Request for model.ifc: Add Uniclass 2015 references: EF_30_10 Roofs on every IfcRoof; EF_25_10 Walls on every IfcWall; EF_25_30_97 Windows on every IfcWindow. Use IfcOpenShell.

First a look at what the model holds.

```python
import ifcopenshell

model = ifcopenshell.open("model.ifc")
print(model.schema)
print("classifications:", [c.Name for c in model.by_type("IfcClassification")])
for ifc_class in ("IfcDoor", "IfcRoof", "IfcStair", "IfcWall", "IfcWindow"):
    print(ifc_class, len(model.by_type(ifc_class)))
```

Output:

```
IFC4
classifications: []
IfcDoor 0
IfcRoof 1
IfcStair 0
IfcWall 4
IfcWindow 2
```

```python
import ifcopenshell
import ifcopenshell.api.classification

model = ifcopenshell.open("model.ifc")

system = ifcopenshell.api.classification.add_classification(model, classification="Uniclass 2015")

codes = {
    "IfcRoof": ("EF_30_10", "Roofs"),
    "IfcWall": ("EF_25_10", "Walls"),
    "IfcWindow": ("EF_25_30_97", "Windows"),
}
for ifc_class, (code, name) in codes.items():
    products = model.by_type(ifc_class)
    ifcopenshell.api.classification.add_reference(
        model, products=products, classification=system, identification=code, name=name
    )
    print(code, len(products))

model.write("model_rev.ifc")
```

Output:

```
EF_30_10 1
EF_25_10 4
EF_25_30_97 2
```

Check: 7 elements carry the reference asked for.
